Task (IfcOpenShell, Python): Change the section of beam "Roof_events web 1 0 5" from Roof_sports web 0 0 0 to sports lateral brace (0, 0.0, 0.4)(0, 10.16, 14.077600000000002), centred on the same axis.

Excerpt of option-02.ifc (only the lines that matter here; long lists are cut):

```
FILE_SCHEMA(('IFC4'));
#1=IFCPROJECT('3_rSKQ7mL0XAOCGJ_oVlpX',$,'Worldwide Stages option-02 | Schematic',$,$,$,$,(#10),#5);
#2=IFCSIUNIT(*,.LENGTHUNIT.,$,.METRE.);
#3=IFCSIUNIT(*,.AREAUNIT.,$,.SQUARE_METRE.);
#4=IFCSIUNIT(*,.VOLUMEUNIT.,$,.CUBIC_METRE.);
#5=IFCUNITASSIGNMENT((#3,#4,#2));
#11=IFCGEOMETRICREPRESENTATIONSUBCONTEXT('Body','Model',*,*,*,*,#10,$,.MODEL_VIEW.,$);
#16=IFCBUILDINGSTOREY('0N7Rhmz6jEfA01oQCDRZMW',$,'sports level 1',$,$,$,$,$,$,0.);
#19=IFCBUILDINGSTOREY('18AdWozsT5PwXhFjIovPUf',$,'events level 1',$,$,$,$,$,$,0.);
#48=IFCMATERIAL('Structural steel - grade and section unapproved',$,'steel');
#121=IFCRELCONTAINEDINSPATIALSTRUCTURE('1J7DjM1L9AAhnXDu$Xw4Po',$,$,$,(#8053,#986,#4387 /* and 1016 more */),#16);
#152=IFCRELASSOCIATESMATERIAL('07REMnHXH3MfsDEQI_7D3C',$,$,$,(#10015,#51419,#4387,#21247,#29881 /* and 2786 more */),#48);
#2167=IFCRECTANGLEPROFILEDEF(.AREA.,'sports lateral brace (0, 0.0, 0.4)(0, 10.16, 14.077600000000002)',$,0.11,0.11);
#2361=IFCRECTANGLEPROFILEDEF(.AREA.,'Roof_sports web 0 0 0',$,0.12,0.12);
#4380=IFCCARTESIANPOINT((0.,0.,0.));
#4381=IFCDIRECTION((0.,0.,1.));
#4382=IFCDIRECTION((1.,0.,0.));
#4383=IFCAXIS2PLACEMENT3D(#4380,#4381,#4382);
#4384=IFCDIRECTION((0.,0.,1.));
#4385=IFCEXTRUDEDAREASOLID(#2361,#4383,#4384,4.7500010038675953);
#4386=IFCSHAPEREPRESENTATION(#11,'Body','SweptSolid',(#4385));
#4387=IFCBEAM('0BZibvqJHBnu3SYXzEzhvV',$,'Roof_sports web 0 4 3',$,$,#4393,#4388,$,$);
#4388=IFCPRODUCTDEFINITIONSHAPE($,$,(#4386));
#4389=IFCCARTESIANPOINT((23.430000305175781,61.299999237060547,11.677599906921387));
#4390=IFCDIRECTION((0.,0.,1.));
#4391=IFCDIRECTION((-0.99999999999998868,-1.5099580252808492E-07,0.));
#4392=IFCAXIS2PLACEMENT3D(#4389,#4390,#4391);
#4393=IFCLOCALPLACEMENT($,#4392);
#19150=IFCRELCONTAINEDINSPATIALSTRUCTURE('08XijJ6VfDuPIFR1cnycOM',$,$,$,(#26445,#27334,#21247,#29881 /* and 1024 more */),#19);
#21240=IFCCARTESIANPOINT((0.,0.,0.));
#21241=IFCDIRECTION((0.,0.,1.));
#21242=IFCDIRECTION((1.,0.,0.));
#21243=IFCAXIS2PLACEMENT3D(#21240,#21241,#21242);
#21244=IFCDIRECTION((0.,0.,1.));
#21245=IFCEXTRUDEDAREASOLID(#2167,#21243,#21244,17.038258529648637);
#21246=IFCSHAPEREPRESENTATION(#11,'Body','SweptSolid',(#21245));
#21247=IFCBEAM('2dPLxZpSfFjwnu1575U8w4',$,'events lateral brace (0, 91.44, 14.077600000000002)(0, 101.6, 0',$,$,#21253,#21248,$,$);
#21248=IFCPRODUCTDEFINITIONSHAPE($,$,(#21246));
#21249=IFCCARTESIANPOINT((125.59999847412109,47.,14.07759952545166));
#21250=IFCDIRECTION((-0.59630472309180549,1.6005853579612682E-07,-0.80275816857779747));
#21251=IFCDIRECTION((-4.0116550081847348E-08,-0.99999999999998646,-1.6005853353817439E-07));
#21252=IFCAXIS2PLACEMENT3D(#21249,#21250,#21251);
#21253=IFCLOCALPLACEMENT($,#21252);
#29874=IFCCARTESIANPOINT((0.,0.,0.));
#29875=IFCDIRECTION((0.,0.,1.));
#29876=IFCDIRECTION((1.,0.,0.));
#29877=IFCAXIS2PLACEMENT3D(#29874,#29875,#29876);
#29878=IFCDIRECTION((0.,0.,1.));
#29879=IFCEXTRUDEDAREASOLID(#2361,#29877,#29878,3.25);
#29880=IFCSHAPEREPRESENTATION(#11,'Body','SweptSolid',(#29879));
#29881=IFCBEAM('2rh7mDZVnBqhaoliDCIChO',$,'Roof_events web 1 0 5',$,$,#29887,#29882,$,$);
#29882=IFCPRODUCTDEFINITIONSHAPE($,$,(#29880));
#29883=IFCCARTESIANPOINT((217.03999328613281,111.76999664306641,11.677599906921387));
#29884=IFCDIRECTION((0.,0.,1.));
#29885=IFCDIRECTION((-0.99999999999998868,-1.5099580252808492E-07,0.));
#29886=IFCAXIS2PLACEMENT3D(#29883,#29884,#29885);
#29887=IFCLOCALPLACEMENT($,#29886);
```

```python
import ifcopenshell
import ifcopenshell.util.element
import ifcopenshell.util.representation

model = ifcopenshell.open("option-02.ifc")

member = model.by_guid("2rh7mDZVnBqhaoliDCIChO")
source = next(p for p in model.by_type("IfcRectangleProfileDef") if p.ProfileName == "sports lateral brace (0, 0.0, 0.4)(0, 10.16, 14.077600000000002)")

body = ifcopenshell.util.representation.get_representation(member, "Model", "Body")
solid = body.Items[0]
old_profile = solid.SweptArea

# Copy the section's sizes but keep this member's own profile position.
profile = ifcopenshell.util.element.copy(model, source)
profile.Position = old_profile.Position
solid.SweptArea = profile
if not model.get_total_inverses(old_profile):
    ifcopenshell.util.element.remove_deep2(model, old_profile)

print(solid.SweptArea)

model.write("option-02-out.ifc")
```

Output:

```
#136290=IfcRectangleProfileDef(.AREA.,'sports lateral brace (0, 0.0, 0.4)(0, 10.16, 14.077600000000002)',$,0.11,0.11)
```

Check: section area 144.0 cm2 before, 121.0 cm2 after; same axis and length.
